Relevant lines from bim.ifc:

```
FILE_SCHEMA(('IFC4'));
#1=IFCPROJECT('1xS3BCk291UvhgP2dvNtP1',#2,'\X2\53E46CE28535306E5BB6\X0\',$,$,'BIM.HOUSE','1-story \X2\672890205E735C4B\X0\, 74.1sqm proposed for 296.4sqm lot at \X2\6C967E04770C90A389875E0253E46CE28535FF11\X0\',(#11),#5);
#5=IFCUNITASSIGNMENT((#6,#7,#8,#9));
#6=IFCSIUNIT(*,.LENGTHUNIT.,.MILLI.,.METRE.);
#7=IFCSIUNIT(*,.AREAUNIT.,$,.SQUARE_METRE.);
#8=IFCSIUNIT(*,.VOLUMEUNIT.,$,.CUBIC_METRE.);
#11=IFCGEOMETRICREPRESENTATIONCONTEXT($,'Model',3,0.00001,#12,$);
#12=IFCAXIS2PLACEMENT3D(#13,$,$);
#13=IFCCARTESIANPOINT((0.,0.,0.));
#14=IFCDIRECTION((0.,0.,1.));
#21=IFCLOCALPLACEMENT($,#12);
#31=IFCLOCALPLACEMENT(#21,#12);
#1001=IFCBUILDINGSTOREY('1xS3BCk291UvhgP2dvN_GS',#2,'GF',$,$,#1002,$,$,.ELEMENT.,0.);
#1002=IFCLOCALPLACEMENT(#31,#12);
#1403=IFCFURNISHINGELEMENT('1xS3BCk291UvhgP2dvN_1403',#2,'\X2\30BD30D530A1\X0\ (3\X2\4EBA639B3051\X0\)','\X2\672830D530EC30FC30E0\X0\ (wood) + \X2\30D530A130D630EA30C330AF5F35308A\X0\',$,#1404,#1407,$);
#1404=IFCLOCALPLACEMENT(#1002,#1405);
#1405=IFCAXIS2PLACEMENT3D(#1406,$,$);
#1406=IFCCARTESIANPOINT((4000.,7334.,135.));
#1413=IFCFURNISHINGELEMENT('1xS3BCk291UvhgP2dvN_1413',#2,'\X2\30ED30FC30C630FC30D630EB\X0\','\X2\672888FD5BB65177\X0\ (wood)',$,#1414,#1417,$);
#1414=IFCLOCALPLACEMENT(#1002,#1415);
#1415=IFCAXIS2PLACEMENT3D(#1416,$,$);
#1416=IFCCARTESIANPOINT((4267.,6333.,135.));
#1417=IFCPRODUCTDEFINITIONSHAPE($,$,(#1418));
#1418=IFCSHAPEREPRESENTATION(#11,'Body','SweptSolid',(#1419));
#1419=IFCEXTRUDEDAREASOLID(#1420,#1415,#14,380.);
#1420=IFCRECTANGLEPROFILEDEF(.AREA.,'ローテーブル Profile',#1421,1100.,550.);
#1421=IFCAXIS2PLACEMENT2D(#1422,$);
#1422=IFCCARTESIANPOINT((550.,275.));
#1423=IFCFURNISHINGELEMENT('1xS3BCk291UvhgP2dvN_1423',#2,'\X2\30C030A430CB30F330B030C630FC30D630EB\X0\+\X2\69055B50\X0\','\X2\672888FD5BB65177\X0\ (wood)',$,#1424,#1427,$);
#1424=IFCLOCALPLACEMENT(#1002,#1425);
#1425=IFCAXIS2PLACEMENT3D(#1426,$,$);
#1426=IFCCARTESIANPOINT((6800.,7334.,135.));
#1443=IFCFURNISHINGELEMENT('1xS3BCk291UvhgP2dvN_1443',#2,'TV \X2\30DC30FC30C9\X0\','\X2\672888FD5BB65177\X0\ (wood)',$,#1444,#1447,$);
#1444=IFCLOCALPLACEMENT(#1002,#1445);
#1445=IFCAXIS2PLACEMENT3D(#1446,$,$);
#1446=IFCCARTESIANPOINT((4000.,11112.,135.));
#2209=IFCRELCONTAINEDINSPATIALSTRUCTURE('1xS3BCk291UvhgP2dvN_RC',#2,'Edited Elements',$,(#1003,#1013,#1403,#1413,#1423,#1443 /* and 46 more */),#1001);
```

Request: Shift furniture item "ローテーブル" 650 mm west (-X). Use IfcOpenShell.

```python
import ifcopenshell
import ifcopenshell.api.geometry
import ifcopenshell.util.placement
import ifcopenshell.util.unit

model = ifcopenshell.open("bim.ifc")
unit_scale = ifcopenshell.util.unit.calculate_unit_scale(model)

item = model.by_id(1413)
matrix = ifcopenshell.util.placement.get_local_placement(item.ObjectPlacement)
matrix[0, 3] -= 0.65 / unit_scale
ifcopenshell.api.geometry.edit_object_placement(model, product=item, matrix=matrix, is_si=False)

print(ifcopenshell.util.placement.get_local_placement(item.ObjectPlacement).round(3) + 0.0)

model.write("bim_rev.ifc")
```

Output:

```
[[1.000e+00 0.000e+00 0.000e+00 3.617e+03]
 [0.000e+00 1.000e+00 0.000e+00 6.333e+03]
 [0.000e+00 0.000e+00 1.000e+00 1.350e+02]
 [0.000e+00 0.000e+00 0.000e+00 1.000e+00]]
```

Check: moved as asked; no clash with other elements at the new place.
